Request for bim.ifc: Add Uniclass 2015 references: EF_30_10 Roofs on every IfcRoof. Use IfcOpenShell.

First a look at what the model holds.

```python
import ifcopenshell

model = ifcopenshell.open("bim.ifc")
print(model.schema)
print("classifications:", [c.Name for c in model.by_type("IfcClassification")])
for ifc_class in ("IfcDoor", "IfcRoof", "IfcStair", "IfcWall", "IfcWindow"):
    print(ifc_class, len(model.by_type(ifc_class)))
```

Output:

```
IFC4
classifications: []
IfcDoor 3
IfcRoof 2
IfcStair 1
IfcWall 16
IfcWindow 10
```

```python
import ifcopenshell
import ifcopenshell.api.classification

model = ifcopenshell.open("bim.ifc")

system = ifcopenshell.api.classification.add_classification(model, classification="Uniclass 2015")

codes = {
    "IfcRoof": ("EF_30_10", "Roofs"),
}
for ifc_class, (code, name) in codes.items():
    products = model.by_type(ifc_class)
    ifcopenshell.api.classification.add_reference(
        model, products=products, classification=system, identification=code, name=name
    )
    print(code, len(products))

model.write("bim_rev.ifc")
```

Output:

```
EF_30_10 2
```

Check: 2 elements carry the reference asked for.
